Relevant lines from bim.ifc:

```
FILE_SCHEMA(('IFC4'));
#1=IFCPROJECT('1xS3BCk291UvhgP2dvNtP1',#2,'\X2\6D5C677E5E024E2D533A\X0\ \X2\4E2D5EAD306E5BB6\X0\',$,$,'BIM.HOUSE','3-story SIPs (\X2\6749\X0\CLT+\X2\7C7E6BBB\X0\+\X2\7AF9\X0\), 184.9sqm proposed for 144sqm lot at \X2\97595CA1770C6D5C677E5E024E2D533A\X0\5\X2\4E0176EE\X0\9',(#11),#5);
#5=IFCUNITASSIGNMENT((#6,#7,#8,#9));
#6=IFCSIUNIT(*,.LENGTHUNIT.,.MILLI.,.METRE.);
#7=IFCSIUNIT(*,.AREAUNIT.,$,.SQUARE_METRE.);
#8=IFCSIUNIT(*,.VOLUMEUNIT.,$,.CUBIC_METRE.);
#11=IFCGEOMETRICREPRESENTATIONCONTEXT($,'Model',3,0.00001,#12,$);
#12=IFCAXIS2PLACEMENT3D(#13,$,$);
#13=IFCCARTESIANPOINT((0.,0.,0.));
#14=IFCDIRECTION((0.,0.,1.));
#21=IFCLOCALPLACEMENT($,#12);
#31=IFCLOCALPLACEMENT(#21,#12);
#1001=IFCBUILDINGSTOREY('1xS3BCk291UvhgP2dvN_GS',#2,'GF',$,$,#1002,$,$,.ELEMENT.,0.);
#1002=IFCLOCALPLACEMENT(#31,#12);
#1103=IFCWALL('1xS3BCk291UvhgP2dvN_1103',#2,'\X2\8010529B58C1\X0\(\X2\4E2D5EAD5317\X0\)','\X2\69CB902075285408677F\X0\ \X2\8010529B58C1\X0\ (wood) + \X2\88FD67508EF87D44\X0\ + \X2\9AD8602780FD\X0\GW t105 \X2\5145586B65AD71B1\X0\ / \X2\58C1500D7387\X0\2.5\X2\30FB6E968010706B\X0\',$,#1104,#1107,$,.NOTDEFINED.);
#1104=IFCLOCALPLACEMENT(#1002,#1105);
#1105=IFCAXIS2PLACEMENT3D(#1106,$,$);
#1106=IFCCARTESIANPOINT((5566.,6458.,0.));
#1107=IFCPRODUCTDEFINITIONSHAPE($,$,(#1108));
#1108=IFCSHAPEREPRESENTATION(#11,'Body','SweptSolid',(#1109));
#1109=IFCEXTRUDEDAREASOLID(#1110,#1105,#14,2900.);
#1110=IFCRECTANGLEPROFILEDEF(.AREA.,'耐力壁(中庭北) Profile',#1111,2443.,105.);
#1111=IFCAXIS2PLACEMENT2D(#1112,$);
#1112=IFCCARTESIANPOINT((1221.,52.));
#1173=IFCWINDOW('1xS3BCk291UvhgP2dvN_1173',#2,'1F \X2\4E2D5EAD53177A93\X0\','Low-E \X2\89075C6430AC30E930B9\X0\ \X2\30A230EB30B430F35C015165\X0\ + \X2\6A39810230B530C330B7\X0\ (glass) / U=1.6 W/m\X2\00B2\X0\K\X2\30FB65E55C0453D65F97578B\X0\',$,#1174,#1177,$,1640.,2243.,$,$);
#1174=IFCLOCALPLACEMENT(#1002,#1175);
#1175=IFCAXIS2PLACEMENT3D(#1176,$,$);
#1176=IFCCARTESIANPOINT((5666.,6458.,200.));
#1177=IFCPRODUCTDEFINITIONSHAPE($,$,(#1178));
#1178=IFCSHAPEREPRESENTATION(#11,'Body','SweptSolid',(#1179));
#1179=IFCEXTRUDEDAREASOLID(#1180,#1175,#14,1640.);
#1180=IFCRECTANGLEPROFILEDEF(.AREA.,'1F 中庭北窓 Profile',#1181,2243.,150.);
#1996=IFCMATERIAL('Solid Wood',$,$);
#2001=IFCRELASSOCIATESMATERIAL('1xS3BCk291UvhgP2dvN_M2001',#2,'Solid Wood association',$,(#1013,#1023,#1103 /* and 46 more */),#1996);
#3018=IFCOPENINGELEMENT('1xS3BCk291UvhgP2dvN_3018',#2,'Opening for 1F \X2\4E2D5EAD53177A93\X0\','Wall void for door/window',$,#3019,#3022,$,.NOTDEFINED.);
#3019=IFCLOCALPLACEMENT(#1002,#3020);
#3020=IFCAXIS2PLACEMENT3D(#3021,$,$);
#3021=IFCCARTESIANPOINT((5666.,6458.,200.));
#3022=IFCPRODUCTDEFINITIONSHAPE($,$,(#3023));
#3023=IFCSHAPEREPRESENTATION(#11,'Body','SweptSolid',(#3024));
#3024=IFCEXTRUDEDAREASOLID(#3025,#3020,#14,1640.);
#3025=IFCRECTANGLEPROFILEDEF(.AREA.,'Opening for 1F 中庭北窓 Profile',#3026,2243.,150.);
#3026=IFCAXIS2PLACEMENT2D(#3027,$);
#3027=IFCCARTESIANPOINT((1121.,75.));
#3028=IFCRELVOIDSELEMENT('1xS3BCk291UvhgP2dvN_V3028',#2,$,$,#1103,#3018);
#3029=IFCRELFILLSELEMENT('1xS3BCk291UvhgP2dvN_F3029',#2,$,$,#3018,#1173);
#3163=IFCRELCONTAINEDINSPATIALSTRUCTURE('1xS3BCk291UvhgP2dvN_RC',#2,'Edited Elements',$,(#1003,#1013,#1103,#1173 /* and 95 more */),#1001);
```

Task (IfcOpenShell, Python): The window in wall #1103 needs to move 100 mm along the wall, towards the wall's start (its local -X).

```python
import ifcopenshell
import ifcopenshell.api.geometry
import ifcopenshell.util.placement
import ifcopenshell.util.unit

model = ifcopenshell.open("bim.ifc")
unit_scale = ifcopenshell.util.unit.calculate_unit_scale(model)

window = model.by_guid("1xS3BCk291UvhgP2dvN_1173")
opening = window.FillsVoids[0].RelatingOpeningElement
wall = opening.VoidsElements[0].RelatingBuildingElement

wall_matrix = ifcopenshell.util.placement.get_local_placement(wall.ObjectPlacement)
shift = wall_matrix[:3, 0] * -0.1 / unit_scale
before = ifcopenshell.util.placement.get_local_placement(window.ObjectPlacement)[:3, 3].copy()

# The window is not placed relative to its opening, so move both.
for product in (opening, window):
    matrix = ifcopenshell.util.placement.get_local_placement(product.ObjectPlacement)
    matrix[:3, 3] += shift
    ifcopenshell.api.geometry.edit_object_placement(model, product=product, matrix=matrix, is_si=False)

after = ifcopenshell.util.placement.get_local_placement(window.ObjectPlacement)[:3, 3]
print("window moved by", (after - before).round(3) + 0.0)

model.write("bim-out.ifc")
```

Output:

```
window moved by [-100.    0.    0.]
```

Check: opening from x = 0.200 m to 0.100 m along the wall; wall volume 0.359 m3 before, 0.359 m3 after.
